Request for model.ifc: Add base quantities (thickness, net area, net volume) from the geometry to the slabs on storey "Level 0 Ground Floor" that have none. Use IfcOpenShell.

First a look at what the model holds.

```python
import ifcopenshell
import ifcopenshell.util.element
import ifcopenshell.util.unit

model = ifcopenshell.open("model.ifc")
print(model.schema)
for unit_type in ("LENGTHUNIT", "AREAUNIT", "VOLUMEUNIT"):
    print(unit_type, ifcopenshell.util.unit.calculate_unit_scale(model, unit_type))
storey = next(s for s in model.by_type("IfcBuildingStorey") if s.Name == "Level 0 Ground Floor")
slabs = [e for e in ifcopenshell.util.element.get_decomposition(storey) if e.is_a("IfcSlab")]
for e in sorted(slabs, key=lambda e: e.id()):
    print(e.id(), e.is_a(), e.Name, list(ifcopenshell.util.element.get_psets(e, qtos_only=True)), sep=" | ")
```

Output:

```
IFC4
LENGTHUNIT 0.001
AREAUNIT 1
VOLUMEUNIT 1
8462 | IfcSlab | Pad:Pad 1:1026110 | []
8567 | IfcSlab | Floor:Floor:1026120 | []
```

```python
import ifcopenshell
import ifcopenshell.api.pset
import ifcopenshell.geom
import ifcopenshell.util.element
import ifcopenshell.util.shape
import ifcopenshell.util.unit

model = ifcopenshell.open("model.ifc")
unit_scale = ifcopenshell.util.unit.calculate_unit_scale(model)
area_scale = ifcopenshell.util.unit.calculate_unit_scale(model, "AREAUNIT")
volume_scale = ifcopenshell.util.unit.calculate_unit_scale(model, "VOLUMEUNIT")
settings = ifcopenshell.geom.settings()

storey = next(s for s in model.by_type("IfcBuildingStorey") if s.Name == "Level 0 Ground Floor")
slabs = [e for e in ifcopenshell.util.element.get_decomposition(storey) if e.is_a("IfcSlab")]

for e in sorted(slabs, key=lambda e: e.id()):
    if ifcopenshell.util.element.get_psets(e, qtos_only=True, should_inherit=False):
        continue
    # Geometry comes back in metres, in the element's own axes.
    shape = ifcopenshell.geom.create_shape(settings, e)
    values = {
        "Width": ifcopenshell.util.shape.get_z(shape.geometry) / unit_scale,
        "NetArea": ifcopenshell.util.shape.get_footprint_area(shape.geometry) / area_scale,
        "NetVolume": ifcopenshell.util.shape.get_volume(shape.geometry) / volume_scale,
    }
    qto = ifcopenshell.api.pset.add_qto(model, product=e, name="Qto_SlabBaseQuantities")
    ifcopenshell.api.pset.edit_qto(model, qto=qto, properties=values)
    print(e.id(), {k: round(v, 3) for k, v in values.items()})

model.write("model_rev.ifc")
```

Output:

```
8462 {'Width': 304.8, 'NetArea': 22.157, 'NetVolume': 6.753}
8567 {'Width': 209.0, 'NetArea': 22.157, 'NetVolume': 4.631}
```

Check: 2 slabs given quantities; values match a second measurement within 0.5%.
